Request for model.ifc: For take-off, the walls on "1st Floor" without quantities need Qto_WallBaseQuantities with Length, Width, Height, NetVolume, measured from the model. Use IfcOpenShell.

First a look at what the model holds.

```python
import ifcopenshell
import ifcopenshell.util.element
import ifcopenshell.util.unit

model = ifcopenshell.open("model.ifc")
print(model.schema)
for unit_type in ("LENGTHUNIT", "AREAUNIT", "VOLUMEUNIT"):
    print(unit_type, ifcopenshell.util.unit.calculate_unit_scale(model, unit_type))
storey = next(s for s in model.by_type("IfcBuildingStorey") if s.Name == "1st Floor")
walls = [e for e in ifcopenshell.util.element.get_decomposition(storey) if e.is_a("IfcWall")]
for e in sorted(walls, key=lambda e: e.id()):
    print(e.id(), e.is_a(), e.Name, list(ifcopenshell.util.element.get_psets(e, qtos_only=True)), sep=" | ")
```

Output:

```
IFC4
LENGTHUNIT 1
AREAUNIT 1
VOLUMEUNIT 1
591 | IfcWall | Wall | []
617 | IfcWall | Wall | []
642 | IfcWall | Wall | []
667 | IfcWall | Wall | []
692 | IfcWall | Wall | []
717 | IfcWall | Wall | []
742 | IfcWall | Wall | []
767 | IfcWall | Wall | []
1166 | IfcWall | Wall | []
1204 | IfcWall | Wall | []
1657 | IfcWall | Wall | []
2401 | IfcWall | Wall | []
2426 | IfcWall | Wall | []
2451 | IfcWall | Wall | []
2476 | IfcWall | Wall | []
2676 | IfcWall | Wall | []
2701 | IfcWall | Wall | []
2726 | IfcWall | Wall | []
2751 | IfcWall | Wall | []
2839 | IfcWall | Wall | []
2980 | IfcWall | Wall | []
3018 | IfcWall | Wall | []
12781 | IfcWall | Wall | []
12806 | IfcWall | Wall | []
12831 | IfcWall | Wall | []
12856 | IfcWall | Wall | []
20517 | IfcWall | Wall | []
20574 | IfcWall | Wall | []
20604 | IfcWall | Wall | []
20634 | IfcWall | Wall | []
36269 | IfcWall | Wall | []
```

```python
import ifcopenshell
import ifcopenshell.api.pset
import ifcopenshell.geom
import ifcopenshell.util.element
import ifcopenshell.util.shape
import ifcopenshell.util.unit

model = ifcopenshell.open("model.ifc")
unit_scale = ifcopenshell.util.unit.calculate_unit_scale(model)
volume_scale = ifcopenshell.util.unit.calculate_unit_scale(model, "VOLUMEUNIT")
settings = ifcopenshell.geom.settings()

storey = next(s for s in model.by_type("IfcBuildingStorey") if s.Name == "1st Floor")
walls = [e for e in ifcopenshell.util.element.get_decomposition(storey) if e.is_a("IfcWall")]

for e in sorted(walls, key=lambda e: e.id()):
    if ifcopenshell.util.element.get_psets(e, qtos_only=True, should_inherit=False):
        continue
    # Geometry comes back in metres, in the element's own axes.
    shape = ifcopenshell.geom.create_shape(settings, e)
    values = {
        "Length": ifcopenshell.util.shape.get_x(shape.geometry) / unit_scale,
        "Width": ifcopenshell.util.shape.get_y(shape.geometry) / unit_scale,
        "Height": ifcopenshell.util.shape.get_z(shape.geometry) / unit_scale,
        "NetVolume": ifcopenshell.util.shape.get_volume(shape.geometry) / volume_scale,
    }
    qto = ifcopenshell.api.pset.add_qto(model, product=e, name="Qto_WallBaseQuantities")
    ifcopenshell.api.pset.edit_qto(model, qto=qto, properties=values)
    print(e.id(), {k: round(v, 3) for k, v in values.items()})

model.write("model-out.ifc")
```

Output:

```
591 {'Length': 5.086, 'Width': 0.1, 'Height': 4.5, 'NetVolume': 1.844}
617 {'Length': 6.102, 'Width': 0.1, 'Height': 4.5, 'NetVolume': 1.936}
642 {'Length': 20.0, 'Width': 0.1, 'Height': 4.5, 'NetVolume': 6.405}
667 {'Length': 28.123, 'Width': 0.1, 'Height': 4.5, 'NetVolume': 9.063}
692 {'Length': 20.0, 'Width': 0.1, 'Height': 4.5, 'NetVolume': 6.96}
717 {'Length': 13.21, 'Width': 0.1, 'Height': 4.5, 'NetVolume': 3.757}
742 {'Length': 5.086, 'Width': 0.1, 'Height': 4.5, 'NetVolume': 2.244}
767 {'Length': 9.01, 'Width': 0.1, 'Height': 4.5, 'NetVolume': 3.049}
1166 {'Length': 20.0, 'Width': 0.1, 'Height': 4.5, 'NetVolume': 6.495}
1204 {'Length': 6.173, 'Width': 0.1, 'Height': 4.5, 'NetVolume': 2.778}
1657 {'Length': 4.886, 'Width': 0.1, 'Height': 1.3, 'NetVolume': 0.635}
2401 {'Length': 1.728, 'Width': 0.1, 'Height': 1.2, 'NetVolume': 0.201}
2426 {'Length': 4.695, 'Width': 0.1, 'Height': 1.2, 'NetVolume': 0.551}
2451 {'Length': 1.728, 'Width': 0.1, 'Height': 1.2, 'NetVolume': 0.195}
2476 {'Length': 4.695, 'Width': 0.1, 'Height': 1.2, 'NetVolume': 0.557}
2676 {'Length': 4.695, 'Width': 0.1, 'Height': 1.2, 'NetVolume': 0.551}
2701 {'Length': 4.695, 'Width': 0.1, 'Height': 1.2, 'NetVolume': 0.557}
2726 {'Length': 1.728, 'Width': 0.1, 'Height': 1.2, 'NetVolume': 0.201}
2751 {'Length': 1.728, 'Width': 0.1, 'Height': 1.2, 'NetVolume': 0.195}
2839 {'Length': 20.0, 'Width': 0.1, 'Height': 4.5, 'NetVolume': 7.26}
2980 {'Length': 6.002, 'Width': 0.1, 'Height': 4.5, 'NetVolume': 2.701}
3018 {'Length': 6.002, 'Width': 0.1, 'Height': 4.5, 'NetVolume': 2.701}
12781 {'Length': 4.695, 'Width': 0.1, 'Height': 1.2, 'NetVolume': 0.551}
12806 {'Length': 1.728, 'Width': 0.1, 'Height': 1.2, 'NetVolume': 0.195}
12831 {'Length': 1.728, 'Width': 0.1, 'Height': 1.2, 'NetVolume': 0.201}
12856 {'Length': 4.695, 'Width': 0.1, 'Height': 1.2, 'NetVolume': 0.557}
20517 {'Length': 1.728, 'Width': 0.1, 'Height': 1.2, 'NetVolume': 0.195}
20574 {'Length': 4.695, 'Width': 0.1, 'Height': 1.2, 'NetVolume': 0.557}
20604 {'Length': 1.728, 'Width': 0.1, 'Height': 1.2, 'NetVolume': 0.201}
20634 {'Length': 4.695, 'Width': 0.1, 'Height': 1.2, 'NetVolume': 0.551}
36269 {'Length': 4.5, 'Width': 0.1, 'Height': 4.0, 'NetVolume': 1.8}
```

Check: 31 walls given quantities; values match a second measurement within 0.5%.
